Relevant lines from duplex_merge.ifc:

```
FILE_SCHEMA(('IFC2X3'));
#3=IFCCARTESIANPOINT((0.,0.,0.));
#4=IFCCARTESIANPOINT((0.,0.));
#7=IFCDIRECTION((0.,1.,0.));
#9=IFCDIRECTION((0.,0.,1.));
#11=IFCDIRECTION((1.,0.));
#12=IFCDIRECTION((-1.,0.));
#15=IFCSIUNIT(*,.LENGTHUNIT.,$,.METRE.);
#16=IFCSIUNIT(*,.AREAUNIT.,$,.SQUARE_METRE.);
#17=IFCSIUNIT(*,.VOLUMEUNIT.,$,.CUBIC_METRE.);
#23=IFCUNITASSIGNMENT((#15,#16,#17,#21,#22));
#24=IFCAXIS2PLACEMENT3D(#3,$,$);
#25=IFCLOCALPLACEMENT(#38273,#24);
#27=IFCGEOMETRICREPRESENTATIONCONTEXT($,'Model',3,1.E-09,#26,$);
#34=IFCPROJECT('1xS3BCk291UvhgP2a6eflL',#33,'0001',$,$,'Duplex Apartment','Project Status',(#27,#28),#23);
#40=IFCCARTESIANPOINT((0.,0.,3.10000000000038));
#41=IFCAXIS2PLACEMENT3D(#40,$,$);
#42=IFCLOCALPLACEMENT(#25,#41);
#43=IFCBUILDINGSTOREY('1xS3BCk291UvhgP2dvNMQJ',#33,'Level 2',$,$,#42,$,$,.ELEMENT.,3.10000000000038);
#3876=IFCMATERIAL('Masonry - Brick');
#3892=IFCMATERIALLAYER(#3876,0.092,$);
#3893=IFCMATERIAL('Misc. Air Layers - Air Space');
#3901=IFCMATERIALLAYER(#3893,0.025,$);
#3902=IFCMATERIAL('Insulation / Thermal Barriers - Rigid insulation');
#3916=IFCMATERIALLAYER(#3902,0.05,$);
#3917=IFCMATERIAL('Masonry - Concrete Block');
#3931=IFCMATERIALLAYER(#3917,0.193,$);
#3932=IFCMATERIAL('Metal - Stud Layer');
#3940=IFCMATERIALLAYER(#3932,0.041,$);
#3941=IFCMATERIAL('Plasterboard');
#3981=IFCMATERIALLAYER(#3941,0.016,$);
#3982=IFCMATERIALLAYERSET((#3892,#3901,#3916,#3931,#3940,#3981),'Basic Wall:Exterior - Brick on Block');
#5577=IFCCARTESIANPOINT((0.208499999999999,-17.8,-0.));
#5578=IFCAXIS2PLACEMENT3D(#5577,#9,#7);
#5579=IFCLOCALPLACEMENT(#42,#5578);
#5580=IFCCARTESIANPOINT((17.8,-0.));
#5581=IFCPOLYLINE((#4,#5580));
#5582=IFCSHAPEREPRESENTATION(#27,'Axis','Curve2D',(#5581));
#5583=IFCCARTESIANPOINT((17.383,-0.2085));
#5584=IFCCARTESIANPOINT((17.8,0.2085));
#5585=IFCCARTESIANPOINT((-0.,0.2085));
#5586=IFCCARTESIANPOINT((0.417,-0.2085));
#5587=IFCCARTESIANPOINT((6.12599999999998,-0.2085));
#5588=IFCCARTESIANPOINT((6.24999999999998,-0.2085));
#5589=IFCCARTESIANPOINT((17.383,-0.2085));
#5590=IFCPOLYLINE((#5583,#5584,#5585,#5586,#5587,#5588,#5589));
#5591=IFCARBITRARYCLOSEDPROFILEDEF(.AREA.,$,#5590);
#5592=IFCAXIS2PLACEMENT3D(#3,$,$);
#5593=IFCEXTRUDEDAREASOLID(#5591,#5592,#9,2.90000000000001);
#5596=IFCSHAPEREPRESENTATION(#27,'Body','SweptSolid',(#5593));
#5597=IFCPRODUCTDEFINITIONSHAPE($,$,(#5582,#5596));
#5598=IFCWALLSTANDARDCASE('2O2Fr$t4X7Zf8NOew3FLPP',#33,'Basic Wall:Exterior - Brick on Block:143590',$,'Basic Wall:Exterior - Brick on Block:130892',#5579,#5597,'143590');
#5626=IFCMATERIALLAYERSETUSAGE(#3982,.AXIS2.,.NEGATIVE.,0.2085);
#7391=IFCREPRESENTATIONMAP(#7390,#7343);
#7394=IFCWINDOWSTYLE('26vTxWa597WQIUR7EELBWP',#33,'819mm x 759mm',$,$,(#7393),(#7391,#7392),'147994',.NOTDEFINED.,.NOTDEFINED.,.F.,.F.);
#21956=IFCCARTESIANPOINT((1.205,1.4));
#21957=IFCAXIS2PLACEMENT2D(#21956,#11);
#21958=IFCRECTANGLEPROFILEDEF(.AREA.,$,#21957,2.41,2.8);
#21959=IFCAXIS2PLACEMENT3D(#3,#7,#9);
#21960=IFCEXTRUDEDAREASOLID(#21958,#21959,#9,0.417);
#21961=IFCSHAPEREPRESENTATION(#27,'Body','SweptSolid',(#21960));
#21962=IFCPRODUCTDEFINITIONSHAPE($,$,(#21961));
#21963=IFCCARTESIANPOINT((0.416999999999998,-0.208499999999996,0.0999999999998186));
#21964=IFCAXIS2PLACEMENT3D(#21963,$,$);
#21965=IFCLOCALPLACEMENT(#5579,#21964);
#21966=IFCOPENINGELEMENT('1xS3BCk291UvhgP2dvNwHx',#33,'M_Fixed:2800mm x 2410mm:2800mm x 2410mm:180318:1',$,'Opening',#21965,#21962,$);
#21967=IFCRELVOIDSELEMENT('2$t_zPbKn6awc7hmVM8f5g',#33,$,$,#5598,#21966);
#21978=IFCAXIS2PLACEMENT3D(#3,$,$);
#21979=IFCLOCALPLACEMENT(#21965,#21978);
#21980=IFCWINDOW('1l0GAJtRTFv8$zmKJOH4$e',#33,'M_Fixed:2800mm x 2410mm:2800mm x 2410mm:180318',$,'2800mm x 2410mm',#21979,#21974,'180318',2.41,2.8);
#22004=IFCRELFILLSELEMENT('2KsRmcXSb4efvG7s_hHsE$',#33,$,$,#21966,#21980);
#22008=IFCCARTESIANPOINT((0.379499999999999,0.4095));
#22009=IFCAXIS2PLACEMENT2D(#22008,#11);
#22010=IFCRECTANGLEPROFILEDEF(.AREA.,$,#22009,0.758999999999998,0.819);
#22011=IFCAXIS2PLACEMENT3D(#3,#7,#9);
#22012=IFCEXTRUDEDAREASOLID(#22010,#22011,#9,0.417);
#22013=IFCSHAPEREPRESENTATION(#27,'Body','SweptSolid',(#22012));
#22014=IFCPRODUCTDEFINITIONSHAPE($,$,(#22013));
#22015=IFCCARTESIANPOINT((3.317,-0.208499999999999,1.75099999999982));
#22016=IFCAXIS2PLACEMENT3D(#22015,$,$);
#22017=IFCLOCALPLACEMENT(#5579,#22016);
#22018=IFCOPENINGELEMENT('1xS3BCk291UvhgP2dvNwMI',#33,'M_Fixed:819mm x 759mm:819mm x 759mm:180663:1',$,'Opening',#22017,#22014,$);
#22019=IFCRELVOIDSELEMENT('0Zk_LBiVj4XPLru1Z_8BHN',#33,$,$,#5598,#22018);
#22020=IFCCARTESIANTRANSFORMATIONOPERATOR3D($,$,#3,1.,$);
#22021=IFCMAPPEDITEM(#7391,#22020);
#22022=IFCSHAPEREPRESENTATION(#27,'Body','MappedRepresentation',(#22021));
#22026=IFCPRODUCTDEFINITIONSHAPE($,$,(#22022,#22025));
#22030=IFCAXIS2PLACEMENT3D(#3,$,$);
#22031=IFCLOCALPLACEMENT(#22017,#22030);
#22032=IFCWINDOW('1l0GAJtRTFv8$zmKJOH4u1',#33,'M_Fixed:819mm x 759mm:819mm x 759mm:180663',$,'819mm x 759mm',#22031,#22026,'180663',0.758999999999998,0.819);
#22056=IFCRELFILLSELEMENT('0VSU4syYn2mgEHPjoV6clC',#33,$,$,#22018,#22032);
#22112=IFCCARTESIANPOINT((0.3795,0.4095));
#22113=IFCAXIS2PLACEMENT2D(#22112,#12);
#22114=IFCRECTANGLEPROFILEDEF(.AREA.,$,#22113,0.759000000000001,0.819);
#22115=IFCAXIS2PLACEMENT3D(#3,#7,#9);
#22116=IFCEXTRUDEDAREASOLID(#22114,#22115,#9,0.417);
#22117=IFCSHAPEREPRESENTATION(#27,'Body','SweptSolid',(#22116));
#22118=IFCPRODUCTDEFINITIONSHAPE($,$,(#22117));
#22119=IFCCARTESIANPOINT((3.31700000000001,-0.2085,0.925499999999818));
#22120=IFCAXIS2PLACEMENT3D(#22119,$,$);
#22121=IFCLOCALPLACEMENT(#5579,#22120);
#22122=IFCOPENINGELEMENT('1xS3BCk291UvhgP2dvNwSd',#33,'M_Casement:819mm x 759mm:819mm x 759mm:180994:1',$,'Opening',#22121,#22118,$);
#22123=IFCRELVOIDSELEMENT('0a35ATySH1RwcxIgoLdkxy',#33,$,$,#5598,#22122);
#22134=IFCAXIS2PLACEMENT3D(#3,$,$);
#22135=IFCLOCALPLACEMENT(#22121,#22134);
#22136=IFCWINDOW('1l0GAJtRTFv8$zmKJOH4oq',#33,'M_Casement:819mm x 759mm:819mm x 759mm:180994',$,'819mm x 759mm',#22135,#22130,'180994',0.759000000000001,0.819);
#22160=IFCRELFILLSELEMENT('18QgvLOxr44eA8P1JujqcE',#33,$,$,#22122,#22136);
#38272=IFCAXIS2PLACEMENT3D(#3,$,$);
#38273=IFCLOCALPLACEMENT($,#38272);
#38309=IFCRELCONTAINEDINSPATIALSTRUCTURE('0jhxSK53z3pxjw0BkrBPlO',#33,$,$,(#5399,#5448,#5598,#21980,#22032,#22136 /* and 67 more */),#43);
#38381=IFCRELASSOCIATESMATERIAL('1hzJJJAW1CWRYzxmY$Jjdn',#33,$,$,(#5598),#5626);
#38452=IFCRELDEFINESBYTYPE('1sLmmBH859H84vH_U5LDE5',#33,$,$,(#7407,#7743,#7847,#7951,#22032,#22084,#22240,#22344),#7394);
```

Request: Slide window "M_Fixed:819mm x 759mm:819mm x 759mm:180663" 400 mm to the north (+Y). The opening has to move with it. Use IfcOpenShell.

```python
import ifcopenshell
import ifcopenshell.api.geometry
import ifcopenshell.util.placement

model = ifcopenshell.open("duplex_merge.ifc")

window = model.by_guid("1l0GAJtRTFv8$zmKJOH4u1")
opening = window.FillsVoids[0].RelatingOpeningElement
wall = opening.VoidsElements[0].RelatingBuildingElement

wall_matrix = ifcopenshell.util.placement.get_local_placement(wall.ObjectPlacement)
shift = wall_matrix[:3, 0] * 0.4
before = ifcopenshell.util.placement.get_local_placement(window.ObjectPlacement)[:3, 3].copy()

# The window is placed relative to its opening, so it follows when the opening moves.
matrix = ifcopenshell.util.placement.get_local_placement(opening.ObjectPlacement)
matrix[:3, 3] += shift
ifcopenshell.api.geometry.edit_object_placement(
    model, product=opening, matrix=matrix, is_si=False, should_transform_children=True
)

after = ifcopenshell.util.placement.get_local_placement(window.ObjectPlacement)[:3, 3]
print("window moved by", (after - before).round(3) + 0.0)

model.write("duplex_merge_v2.ifc")
```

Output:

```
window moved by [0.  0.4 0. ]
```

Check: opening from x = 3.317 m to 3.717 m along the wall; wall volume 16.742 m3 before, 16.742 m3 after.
